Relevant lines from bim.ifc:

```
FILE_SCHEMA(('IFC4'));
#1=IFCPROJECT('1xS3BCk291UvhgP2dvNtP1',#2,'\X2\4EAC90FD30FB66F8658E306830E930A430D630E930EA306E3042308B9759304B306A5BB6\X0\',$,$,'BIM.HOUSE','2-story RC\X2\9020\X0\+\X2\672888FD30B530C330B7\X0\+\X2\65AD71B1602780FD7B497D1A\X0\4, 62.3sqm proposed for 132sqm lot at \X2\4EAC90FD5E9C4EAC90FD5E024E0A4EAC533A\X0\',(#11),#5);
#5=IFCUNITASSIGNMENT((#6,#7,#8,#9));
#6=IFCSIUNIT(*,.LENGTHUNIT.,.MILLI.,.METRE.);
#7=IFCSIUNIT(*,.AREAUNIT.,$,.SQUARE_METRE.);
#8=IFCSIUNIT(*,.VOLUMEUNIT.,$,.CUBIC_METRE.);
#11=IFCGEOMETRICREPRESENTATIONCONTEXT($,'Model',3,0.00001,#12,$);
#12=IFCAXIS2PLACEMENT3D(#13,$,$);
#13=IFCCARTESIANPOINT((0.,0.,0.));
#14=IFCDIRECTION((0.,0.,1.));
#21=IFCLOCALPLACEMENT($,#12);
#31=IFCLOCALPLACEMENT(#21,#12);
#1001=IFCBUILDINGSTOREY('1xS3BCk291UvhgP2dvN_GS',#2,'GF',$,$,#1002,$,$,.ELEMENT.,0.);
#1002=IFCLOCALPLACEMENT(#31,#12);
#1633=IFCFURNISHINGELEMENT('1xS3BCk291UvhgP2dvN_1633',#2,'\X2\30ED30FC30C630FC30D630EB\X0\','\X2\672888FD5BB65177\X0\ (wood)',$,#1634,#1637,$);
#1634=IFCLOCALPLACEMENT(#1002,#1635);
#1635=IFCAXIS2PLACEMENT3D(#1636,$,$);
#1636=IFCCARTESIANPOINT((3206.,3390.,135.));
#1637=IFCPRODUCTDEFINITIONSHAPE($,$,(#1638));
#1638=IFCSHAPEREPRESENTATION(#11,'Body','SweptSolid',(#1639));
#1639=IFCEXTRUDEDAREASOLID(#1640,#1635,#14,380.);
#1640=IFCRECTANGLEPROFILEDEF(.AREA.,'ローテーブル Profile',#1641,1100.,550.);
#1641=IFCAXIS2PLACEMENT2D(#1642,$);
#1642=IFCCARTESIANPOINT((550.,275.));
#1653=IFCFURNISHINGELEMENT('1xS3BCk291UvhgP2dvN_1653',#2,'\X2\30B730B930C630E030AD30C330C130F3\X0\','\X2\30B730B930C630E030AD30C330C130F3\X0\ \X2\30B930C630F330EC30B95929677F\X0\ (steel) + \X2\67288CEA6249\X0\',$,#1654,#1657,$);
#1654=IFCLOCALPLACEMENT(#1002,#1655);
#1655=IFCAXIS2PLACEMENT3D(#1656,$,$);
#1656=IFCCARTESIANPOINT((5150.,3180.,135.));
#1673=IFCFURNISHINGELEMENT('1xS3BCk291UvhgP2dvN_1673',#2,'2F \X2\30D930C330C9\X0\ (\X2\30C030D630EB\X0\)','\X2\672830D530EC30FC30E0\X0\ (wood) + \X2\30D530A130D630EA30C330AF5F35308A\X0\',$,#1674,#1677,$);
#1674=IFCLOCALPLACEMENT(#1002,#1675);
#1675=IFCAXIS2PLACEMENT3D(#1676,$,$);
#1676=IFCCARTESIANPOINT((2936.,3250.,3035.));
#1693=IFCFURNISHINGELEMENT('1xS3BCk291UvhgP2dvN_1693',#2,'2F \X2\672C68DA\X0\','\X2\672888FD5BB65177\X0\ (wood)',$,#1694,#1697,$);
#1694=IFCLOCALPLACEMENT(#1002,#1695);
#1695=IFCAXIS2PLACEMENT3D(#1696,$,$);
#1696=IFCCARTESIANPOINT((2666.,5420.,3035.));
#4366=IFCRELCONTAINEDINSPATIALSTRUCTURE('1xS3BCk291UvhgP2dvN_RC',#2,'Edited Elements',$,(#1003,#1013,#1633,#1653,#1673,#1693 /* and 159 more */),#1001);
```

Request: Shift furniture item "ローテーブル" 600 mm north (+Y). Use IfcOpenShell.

```python
import ifcopenshell
import ifcopenshell.api.geometry
import ifcopenshell.util.placement
import ifcopenshell.util.unit

model = ifcopenshell.open("bim.ifc")
unit_scale = ifcopenshell.util.unit.calculate_unit_scale(model)

item = model.by_guid("1xS3BCk291UvhgP2dvN_1633")
matrix = ifcopenshell.util.placement.get_local_placement(item.ObjectPlacement)
matrix[1, 3] += 0.6 / unit_scale
ifcopenshell.api.geometry.edit_object_placement(model, product=item, matrix=matrix, is_si=False)

print(ifcopenshell.util.placement.get_local_placement(item.ObjectPlacement).round(3) + 0.0)

model.write("bim_rev.ifc")
```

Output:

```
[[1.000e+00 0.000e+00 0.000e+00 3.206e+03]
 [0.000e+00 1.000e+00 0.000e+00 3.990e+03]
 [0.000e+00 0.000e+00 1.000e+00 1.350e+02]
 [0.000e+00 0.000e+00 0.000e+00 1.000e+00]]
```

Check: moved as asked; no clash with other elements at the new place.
